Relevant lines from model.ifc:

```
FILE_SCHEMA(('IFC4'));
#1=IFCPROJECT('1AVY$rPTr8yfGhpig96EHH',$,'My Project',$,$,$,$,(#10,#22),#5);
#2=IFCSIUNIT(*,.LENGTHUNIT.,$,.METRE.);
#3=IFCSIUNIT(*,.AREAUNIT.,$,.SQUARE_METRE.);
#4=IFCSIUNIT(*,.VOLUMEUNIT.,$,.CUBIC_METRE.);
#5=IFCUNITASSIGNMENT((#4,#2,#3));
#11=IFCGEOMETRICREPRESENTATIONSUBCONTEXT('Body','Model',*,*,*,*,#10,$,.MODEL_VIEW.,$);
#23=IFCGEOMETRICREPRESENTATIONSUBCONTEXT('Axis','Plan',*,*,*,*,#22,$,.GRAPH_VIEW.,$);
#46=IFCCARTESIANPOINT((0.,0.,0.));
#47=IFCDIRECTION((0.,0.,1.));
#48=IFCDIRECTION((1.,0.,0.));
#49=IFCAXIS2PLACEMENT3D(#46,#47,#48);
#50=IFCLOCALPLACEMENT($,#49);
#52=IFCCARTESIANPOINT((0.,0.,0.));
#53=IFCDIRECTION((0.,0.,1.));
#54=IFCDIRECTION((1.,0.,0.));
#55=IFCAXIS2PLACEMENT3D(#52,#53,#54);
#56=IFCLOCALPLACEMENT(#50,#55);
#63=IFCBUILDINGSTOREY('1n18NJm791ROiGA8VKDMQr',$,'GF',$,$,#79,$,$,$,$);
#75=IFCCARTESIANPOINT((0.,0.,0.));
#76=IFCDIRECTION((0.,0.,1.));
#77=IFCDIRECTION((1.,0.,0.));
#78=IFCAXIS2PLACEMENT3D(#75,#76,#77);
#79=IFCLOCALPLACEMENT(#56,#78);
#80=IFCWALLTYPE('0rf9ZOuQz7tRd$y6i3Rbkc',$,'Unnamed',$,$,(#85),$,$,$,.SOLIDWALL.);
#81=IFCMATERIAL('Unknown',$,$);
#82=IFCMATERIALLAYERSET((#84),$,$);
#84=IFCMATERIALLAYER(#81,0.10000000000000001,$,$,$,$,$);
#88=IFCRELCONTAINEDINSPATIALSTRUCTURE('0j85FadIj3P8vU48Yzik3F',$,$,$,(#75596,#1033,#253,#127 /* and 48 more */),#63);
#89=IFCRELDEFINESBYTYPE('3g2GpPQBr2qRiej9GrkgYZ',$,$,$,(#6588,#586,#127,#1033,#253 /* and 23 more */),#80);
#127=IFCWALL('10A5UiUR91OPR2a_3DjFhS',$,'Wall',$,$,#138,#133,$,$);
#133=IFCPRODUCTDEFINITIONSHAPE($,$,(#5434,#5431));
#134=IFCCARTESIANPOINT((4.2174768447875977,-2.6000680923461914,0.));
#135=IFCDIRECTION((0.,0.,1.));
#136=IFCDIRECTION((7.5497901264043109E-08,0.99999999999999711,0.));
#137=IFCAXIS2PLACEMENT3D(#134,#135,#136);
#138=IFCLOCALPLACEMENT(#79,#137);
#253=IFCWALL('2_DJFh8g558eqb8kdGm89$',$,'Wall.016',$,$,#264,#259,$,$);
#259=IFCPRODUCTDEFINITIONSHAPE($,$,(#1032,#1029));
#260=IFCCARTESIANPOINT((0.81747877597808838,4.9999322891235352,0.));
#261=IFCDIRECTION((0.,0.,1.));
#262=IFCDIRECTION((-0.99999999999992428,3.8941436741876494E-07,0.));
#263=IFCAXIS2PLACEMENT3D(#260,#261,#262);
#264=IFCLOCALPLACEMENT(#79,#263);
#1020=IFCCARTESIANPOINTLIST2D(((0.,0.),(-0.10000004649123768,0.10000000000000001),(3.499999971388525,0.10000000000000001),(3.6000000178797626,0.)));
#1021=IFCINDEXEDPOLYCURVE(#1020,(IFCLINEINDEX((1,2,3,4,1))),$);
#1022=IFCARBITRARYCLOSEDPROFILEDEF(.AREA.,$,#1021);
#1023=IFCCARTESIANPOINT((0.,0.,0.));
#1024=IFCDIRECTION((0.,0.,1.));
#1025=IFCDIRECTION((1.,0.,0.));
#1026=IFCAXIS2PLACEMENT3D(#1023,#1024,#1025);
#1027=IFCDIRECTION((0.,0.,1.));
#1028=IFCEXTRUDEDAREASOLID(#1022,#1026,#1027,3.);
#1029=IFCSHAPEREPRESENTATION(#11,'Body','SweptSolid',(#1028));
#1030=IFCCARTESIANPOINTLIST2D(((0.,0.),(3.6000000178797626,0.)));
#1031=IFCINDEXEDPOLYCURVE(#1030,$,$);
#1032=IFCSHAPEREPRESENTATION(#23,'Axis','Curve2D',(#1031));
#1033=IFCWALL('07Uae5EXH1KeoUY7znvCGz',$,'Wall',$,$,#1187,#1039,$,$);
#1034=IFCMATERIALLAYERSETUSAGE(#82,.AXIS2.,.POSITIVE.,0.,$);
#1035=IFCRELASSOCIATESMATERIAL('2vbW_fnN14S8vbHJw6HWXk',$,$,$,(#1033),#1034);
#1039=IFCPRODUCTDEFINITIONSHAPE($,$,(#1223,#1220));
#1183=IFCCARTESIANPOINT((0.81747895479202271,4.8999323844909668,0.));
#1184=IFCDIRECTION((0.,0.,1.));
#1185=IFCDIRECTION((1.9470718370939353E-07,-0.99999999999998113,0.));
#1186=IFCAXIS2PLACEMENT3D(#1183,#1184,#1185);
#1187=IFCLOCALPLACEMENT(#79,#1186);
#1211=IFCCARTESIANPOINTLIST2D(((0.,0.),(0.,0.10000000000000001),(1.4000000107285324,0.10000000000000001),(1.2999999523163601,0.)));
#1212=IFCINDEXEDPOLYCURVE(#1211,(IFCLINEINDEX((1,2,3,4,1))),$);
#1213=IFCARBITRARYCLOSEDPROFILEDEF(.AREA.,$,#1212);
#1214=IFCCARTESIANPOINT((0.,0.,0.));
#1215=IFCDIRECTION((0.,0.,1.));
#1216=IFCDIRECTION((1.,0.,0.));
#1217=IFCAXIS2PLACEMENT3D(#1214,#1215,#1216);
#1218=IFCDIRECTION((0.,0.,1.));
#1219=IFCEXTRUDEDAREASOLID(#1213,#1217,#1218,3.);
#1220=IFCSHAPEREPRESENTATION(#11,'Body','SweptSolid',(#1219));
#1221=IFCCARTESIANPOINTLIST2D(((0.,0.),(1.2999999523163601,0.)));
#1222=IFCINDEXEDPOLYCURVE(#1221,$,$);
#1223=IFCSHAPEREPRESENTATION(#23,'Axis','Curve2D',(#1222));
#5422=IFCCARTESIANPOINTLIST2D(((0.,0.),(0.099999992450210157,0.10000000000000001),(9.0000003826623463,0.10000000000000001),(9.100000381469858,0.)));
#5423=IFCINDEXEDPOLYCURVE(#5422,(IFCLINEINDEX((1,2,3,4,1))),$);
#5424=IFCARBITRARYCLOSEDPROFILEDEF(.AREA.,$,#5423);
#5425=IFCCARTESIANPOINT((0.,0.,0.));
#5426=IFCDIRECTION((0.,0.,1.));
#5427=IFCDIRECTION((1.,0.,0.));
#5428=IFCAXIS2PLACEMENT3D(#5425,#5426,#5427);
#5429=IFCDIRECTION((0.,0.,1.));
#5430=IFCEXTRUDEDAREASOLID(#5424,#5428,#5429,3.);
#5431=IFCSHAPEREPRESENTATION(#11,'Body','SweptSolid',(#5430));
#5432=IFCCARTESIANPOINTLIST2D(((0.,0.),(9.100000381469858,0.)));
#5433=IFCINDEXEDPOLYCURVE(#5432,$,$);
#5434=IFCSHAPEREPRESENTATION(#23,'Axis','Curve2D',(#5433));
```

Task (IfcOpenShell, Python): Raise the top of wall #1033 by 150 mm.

```python
import ifcopenshell
import ifcopenshell.geom
import ifcopenshell.util.representation
import ifcopenshell.util.shape
import ifcopenshell.util.unit

model = ifcopenshell.open("model.ifc")
unit_scale = ifcopenshell.util.unit.calculate_unit_scale(model)
settings = ifcopenshell.geom.settings()


def volume(element):
    """Net volume in cubic metres, openings subtracted."""
    shape = ifcopenshell.geom.create_shape(settings, element)
    return ifcopenshell.util.shape.get_volume(shape.geometry)


wall = model.by_guid("07Uae5EXH1KeoUY7znvCGz")
before = volume(wall)

body = ifcopenshell.util.representation.get_representation(wall, "Model", "Body")
solid = body.Items[0]
old_height = solid.Depth
solid.Depth += 0.15 / unit_scale
after = volume(wall)

print(f"height {old_height:g} -> {solid.Depth:g}, volume {before:.3f} -> {after:.3f} m3")

model.write("model_updated.ifc")
```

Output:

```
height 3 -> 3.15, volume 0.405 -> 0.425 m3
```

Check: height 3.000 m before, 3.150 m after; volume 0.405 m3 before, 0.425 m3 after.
